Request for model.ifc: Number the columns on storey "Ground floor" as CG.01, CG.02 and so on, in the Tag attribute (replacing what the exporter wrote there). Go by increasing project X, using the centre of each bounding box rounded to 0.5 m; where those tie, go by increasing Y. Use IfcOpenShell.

First a look at what the model holds.

```python
import ifcopenshell
import ifcopenshell.util.element
import ifcopenshell.util.placement

model = ifcopenshell.open("model.ifc")
print(model.schema)
storey = next(s for s in model.by_type("IfcBuildingStorey") if s.Name == "Ground floor")
columns = [e for e in ifcopenshell.util.element.get_decomposition(storey) if e.is_a("IfcColumn")]
for e in sorted(columns, key=lambda e: e.id()):
    origin = ifcopenshell.util.placement.get_local_placement(e.ObjectPlacement)[:3, 3]
    print(e.id(), e.Tag, e.Name, origin.round(2) + 0.0, sep=" | ")
```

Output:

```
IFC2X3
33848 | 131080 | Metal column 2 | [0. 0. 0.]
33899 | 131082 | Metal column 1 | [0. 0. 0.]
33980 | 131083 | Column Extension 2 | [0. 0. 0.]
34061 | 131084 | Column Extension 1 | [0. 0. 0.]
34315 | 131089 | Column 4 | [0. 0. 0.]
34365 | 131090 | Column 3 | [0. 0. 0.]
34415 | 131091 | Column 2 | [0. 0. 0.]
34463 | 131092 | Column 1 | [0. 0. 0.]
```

```python
import ifcopenshell
import ifcopenshell.geom
import ifcopenshell.util.element
import ifcopenshell.util.shape

model = ifcopenshell.open("model.ifc")
settings = ifcopenshell.geom.settings()
settings.set("use-world-coords", True)


def centre(element):
    shape = ifcopenshell.geom.create_shape(settings, element)
    return ifcopenshell.util.shape.get_bbox_centroid(shape.geometry)


storey = next(s for s in model.by_type("IfcBuildingStorey") if s.Name == "Ground floor")
columns = [e for e in ifcopenshell.util.element.get_decomposition(storey) if e.is_a("IfcColumn")]

# Insertion points can sit at a corner or the storey origin, so sort by the geometry (in metres).
centres = {e: centre(e) for e in columns}
columns.sort(key=lambda e: (round(centres[e][0] / 0.5), centres[e][1]))

for i, e in enumerate(columns, start=1):
    number = f"CG.{i:02d}"
    e.Tag = number
    print(e.id(), number)

model.write("model_v2.ifc")
```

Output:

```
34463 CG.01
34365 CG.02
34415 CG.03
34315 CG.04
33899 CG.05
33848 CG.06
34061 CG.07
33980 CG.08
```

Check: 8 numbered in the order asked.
